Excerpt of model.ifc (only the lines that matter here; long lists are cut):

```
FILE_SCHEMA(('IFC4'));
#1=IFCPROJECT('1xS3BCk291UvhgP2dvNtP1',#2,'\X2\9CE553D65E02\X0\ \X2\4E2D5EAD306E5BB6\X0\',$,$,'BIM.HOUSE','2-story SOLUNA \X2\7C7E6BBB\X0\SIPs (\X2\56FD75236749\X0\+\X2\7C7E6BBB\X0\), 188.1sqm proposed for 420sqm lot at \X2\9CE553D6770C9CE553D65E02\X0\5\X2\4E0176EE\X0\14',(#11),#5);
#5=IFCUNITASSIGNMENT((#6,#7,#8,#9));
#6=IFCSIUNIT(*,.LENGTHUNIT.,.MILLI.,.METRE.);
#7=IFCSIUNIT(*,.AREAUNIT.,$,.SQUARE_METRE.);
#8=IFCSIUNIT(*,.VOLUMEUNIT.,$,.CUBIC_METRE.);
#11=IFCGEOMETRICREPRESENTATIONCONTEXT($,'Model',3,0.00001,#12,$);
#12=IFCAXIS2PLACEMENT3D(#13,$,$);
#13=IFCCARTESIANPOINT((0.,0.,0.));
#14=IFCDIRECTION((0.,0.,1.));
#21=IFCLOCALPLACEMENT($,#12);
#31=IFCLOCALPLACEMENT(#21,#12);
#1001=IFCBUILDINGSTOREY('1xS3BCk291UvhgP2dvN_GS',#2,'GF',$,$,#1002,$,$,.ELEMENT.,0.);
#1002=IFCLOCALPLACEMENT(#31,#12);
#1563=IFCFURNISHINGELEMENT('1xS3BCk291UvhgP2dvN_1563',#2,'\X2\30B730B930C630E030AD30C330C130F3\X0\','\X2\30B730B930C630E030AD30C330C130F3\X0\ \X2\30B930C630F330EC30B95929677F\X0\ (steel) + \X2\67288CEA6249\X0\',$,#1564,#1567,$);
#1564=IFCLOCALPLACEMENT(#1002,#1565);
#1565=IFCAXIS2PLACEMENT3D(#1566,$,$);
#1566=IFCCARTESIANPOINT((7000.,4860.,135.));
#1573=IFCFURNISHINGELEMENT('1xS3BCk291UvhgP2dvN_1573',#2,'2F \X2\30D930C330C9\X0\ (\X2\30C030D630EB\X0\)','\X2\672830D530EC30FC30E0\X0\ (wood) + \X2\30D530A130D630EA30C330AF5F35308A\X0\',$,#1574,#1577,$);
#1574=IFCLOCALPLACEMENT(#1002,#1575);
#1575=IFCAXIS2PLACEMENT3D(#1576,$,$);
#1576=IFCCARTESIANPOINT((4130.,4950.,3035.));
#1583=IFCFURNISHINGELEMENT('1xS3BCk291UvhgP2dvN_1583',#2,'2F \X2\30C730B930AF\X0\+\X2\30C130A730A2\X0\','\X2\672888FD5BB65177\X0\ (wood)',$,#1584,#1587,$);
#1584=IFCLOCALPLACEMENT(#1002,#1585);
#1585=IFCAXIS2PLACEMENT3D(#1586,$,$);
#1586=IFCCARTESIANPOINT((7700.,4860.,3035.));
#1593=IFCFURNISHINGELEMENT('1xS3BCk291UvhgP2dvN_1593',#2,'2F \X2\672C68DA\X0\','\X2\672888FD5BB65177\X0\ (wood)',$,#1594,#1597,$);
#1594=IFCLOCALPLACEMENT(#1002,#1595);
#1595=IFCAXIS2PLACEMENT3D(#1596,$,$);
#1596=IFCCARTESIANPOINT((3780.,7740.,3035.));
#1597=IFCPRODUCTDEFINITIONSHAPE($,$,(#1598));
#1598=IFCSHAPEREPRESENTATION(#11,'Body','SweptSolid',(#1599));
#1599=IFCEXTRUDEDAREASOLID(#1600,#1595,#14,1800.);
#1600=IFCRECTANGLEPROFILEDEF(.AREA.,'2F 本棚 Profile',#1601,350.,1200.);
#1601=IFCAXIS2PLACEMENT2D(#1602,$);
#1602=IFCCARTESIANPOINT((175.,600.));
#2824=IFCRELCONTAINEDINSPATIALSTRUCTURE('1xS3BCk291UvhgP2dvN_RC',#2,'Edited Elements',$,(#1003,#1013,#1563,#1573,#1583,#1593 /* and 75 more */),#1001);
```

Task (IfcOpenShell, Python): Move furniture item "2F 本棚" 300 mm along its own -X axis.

```python
import ifcopenshell
import ifcopenshell.api.geometry
import ifcopenshell.util.placement
import ifcopenshell.util.unit

model = ifcopenshell.open("model.ifc")
unit_scale = ifcopenshell.util.unit.calculate_unit_scale(model)

item = model.by_guid("1xS3BCk291UvhgP2dvN_1593")
matrix = ifcopenshell.util.placement.get_local_placement(item.ObjectPlacement)
matrix[:3, 3] -= matrix[:3, 0] * 0.3 / unit_scale
ifcopenshell.api.geometry.edit_object_placement(model, product=item, matrix=matrix, is_si=False)

print(ifcopenshell.util.placement.get_local_placement(item.ObjectPlacement).round(3) + 0.0)

model.write("model_v2.ifc")
```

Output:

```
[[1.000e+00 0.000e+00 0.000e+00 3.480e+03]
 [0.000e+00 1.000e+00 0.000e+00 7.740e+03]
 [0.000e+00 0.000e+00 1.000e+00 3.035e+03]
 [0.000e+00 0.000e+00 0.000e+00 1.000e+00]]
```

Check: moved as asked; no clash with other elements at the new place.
